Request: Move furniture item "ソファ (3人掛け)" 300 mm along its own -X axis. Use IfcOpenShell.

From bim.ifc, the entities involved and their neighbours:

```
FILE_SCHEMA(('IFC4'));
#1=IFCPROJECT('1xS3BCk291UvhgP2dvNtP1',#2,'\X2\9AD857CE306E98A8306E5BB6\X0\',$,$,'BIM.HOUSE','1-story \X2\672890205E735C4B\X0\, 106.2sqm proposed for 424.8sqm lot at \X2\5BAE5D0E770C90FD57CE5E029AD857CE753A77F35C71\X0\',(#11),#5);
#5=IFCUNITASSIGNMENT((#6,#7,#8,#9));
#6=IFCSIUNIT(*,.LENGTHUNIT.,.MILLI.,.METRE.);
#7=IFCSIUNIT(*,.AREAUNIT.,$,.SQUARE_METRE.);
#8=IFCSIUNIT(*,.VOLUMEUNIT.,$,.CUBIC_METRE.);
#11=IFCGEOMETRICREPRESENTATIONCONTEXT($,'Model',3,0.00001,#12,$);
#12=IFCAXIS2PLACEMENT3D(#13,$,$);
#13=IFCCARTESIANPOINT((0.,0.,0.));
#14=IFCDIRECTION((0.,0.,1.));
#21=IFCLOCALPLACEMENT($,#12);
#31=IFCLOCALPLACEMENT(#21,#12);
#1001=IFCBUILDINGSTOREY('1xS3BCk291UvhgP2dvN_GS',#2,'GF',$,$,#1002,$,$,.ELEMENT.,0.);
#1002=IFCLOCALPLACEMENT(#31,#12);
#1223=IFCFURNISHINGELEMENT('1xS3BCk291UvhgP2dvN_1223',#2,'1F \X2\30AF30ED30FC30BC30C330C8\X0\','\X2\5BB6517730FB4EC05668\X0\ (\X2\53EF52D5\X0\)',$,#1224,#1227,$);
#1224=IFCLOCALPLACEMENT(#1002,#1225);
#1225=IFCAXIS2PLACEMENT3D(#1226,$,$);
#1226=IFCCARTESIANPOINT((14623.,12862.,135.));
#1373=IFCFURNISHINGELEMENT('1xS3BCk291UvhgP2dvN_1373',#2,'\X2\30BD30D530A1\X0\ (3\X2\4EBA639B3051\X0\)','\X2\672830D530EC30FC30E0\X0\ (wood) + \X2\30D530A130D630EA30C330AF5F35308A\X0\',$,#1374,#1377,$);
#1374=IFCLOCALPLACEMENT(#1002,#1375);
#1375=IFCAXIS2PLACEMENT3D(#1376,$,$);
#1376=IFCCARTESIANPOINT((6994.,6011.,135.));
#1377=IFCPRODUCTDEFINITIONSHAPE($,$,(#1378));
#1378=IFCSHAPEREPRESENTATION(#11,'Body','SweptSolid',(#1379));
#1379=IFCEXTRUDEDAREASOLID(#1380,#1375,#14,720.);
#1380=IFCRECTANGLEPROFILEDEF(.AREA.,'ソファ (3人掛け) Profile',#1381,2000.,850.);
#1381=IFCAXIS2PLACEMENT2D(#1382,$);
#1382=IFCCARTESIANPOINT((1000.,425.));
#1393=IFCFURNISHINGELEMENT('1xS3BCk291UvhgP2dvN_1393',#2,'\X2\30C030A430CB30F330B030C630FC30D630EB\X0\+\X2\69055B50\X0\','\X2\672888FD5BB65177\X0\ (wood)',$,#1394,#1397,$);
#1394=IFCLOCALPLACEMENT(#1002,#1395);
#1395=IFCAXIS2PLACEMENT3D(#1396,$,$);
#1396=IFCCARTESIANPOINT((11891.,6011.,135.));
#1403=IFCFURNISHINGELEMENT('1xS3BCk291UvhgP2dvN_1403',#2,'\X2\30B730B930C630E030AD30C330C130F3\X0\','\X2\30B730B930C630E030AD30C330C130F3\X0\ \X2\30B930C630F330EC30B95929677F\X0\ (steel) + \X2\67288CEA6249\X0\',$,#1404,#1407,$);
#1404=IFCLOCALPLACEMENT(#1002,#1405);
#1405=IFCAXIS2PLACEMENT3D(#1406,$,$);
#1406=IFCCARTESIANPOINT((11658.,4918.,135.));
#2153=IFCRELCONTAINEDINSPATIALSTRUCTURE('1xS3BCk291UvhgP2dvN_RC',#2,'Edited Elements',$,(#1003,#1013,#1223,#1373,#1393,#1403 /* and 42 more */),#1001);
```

```python
import ifcopenshell
import ifcopenshell.api.geometry
import ifcopenshell.util.placement

model = ifcopenshell.open("bim.ifc")

item = model.by_guid("1xS3BCk291UvhgP2dvN_1373")
matrix = ifcopenshell.util.placement.get_local_placement(item.ObjectPlacement)
matrix[:3, 3] -= matrix[:3, 0] * 300.0
ifcopenshell.api.geometry.edit_object_placement(model, product=item, matrix=matrix, is_si=False)

print(ifcopenshell.util.placement.get_local_placement(item.ObjectPlacement).round(3) + 0.0)

model.write("bim_rev.ifc")
```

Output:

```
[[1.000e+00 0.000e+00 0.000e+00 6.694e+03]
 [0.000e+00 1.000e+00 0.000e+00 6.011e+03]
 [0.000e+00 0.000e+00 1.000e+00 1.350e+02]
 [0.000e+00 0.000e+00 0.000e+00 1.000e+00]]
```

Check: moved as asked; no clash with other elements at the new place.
